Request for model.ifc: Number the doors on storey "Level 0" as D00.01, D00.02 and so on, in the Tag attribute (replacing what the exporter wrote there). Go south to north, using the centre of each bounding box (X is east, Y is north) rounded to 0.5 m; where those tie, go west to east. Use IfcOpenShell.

First a look at what the model holds.

```python
import ifcopenshell
import ifcopenshell.util.element
import ifcopenshell.util.placement

model = ifcopenshell.open("model.ifc")
print(model.schema)
storey = next(s for s in model.by_type("IfcBuildingStorey") if s.Name == "Level 0")
doors = [e for e in ifcopenshell.util.element.get_decomposition(storey) if e.is_a("IfcDoor")]
for e in sorted(doors, key=lambda e: e.id()):
    origin = ifcopenshell.util.placement.get_local_placement(e.ObjectPlacement)[:3, 3]
    print(e.id(), e.Tag, e.Name, origin.round(2) + 0.0, sep=" | ")
```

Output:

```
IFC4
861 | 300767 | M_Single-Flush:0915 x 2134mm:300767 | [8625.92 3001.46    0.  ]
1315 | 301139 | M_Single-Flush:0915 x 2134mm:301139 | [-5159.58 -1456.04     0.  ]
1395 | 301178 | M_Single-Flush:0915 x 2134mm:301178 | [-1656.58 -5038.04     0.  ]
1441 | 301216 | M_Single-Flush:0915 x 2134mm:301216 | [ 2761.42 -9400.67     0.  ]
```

```python
import ifcopenshell
import ifcopenshell.geom
import ifcopenshell.util.element
import ifcopenshell.util.shape

model = ifcopenshell.open("model.ifc")
settings = ifcopenshell.geom.settings()
settings.set("use-world-coords", True)


def centre(element):
    shape = ifcopenshell.geom.create_shape(settings, element)
    return ifcopenshell.util.shape.get_bbox_centroid(shape.geometry)


storey = next(s for s in model.by_type("IfcBuildingStorey") if s.Name == "Level 0")
doors = [e for e in ifcopenshell.util.element.get_decomposition(storey) if e.is_a("IfcDoor")]

# Insertion points can sit at a corner or the storey origin, so sort by the geometry (in metres).
centres = {e: centre(e) for e in doors}
doors.sort(key=lambda e: (round(centres[e][1] / 0.5), centres[e][0]))

for i, e in enumerate(doors, start=1):
    number = f"D00.{i:02d}"
    e.Tag = number
    print(e.id(), number)

model.write("model_v2.ifc")
```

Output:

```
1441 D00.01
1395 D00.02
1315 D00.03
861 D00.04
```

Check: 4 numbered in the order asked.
